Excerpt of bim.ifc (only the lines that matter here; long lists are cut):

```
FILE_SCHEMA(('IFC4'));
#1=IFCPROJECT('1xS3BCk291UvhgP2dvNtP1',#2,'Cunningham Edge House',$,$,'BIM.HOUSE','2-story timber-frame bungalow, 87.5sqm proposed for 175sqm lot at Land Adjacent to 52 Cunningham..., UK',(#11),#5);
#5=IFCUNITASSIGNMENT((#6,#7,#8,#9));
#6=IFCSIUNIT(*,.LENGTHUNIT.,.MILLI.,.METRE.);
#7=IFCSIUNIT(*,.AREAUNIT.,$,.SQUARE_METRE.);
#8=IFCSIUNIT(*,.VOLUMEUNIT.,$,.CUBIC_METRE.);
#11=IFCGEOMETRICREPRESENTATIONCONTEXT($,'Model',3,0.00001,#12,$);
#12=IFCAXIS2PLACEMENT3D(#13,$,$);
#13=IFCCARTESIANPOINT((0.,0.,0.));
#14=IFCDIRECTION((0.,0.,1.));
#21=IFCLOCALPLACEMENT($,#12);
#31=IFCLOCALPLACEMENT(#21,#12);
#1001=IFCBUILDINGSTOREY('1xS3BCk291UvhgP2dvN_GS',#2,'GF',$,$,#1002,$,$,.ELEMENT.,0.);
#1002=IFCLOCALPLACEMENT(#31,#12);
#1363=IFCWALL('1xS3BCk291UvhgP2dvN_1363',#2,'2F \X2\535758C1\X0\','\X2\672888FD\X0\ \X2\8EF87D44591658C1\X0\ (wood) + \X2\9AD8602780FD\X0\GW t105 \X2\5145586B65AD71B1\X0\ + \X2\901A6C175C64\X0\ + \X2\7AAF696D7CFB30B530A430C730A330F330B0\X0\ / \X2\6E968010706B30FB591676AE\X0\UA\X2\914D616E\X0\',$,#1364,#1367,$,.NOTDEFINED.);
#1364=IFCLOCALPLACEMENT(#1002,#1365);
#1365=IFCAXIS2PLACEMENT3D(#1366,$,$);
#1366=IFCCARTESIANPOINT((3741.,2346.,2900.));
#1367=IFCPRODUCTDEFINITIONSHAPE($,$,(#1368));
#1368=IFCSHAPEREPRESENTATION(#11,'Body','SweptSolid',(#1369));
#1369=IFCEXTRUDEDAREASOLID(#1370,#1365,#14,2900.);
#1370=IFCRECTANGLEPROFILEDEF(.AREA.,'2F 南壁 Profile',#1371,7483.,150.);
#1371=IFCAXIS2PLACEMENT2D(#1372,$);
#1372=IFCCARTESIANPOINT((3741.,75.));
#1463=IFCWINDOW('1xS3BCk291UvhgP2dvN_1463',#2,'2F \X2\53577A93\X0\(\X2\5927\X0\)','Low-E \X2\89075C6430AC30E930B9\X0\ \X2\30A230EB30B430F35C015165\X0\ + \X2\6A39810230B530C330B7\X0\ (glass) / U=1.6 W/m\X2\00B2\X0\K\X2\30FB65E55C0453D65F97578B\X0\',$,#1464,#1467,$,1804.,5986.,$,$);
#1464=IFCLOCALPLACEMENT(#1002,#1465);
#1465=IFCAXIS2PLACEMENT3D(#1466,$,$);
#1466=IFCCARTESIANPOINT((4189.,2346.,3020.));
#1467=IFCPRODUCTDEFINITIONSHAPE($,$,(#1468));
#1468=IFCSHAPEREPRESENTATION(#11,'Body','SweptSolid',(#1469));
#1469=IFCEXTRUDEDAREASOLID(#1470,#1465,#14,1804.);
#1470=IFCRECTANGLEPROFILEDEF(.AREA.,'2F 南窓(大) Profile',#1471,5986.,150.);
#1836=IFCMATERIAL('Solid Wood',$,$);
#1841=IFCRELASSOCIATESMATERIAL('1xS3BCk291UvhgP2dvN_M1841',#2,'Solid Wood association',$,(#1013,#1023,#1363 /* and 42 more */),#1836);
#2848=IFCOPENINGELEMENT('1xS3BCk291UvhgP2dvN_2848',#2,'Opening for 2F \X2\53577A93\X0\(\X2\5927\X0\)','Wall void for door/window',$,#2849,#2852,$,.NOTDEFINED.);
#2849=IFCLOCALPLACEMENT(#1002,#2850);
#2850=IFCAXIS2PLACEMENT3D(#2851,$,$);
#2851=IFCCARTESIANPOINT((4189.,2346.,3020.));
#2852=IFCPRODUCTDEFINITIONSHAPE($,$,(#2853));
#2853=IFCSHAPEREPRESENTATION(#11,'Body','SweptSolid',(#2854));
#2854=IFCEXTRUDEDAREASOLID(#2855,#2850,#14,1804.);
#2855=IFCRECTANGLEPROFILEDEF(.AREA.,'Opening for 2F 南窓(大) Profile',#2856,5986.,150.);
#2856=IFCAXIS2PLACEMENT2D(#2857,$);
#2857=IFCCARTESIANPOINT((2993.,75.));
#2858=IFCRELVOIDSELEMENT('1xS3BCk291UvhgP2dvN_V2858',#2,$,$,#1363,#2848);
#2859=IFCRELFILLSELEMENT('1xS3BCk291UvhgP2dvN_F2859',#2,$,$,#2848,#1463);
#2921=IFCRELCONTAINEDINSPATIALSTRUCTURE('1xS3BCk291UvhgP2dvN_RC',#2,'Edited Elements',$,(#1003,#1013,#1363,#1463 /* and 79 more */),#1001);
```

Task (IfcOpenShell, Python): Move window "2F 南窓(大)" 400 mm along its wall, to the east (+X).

```python
import ifcopenshell
import ifcopenshell.api.geometry
import ifcopenshell.util.placement
import ifcopenshell.util.unit

model = ifcopenshell.open("bim.ifc")
unit_scale = ifcopenshell.util.unit.calculate_unit_scale(model)

window = model.by_guid("1xS3BCk291UvhgP2dvN_1463")
opening = window.FillsVoids[0].RelatingOpeningElement
wall = opening.VoidsElements[0].RelatingBuildingElement

wall_matrix = ifcopenshell.util.placement.get_local_placement(wall.ObjectPlacement)
shift = wall_matrix[:3, 0] * 0.4 / unit_scale
before = ifcopenshell.util.placement.get_local_placement(window.ObjectPlacement)[:3, 3].copy()

# The window is not placed relative to its opening, so move both.
for product in (opening, window):
    matrix = ifcopenshell.util.placement.get_local_placement(product.ObjectPlacement)
    matrix[:3, 3] += shift
    ifcopenshell.api.geometry.edit_object_placement(model, product=product, matrix=matrix, is_si=False)

after = ifcopenshell.util.placement.get_local_placement(window.ObjectPlacement)[:3, 3]
print("window moved by", (after - before).round(3) + 0.0)

model.write("bim_updated.ifc")
```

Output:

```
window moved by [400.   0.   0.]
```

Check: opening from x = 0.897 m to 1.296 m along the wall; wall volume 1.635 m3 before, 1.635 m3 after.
